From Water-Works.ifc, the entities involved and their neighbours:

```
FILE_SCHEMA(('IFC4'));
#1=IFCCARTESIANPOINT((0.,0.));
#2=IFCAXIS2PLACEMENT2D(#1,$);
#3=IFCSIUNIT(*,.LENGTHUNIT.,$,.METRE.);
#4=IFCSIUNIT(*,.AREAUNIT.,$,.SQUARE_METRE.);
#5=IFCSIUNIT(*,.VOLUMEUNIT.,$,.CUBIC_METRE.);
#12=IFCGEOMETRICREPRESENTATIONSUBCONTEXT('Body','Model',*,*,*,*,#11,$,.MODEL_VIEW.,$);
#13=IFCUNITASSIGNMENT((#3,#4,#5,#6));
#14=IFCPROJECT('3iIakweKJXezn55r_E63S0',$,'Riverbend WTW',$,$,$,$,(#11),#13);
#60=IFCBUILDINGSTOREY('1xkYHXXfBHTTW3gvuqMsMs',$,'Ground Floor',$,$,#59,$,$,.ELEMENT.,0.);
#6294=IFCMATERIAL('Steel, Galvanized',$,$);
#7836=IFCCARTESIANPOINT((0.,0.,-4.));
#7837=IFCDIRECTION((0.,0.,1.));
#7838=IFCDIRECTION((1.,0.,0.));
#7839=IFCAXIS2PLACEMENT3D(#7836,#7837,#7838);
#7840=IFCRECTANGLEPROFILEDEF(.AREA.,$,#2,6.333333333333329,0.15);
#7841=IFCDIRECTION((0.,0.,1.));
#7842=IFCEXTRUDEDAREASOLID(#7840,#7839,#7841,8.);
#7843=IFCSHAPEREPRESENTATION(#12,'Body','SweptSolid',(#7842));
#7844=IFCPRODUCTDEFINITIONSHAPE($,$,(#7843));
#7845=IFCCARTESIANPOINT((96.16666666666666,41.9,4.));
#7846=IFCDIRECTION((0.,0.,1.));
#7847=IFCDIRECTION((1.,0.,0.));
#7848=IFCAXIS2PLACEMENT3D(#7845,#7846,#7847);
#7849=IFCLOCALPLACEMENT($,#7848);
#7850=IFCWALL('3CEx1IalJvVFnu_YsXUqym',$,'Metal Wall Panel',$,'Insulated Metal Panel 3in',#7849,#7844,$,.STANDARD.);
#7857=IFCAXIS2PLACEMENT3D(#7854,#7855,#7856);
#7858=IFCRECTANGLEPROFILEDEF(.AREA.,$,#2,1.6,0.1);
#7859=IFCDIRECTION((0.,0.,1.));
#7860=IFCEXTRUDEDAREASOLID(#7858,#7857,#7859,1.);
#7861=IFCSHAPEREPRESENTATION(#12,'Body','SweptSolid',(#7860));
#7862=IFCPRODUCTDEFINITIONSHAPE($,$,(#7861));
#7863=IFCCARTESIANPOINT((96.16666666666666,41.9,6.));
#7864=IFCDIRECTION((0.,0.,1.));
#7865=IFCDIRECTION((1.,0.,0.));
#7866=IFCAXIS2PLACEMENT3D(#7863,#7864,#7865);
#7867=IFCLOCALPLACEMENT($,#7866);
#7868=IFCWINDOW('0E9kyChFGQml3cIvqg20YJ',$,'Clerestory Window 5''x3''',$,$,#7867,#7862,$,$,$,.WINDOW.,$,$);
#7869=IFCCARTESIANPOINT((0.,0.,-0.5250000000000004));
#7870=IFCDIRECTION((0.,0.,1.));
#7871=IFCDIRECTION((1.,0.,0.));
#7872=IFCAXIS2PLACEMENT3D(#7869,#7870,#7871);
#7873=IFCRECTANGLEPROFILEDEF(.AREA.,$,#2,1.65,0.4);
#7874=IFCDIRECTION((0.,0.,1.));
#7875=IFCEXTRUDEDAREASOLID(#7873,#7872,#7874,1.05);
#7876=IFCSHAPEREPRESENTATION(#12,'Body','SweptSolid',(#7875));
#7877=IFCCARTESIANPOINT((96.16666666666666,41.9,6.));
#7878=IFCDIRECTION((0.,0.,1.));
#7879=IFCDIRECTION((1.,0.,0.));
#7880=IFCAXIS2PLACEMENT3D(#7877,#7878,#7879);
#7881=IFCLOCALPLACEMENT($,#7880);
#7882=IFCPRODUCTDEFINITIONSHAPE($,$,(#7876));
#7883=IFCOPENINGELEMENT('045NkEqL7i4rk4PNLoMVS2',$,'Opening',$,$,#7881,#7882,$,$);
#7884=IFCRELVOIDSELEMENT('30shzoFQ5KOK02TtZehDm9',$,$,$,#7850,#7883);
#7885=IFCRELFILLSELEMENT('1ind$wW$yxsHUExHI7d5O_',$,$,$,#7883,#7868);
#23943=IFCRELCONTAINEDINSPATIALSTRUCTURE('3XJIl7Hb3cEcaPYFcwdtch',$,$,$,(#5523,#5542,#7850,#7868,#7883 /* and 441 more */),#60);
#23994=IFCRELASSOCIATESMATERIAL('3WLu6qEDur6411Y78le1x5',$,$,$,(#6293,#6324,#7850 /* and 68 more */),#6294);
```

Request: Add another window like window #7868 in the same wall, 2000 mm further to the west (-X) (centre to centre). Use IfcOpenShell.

```python
import ifcopenshell
import ifcopenshell.api.feature
import ifcopenshell.api.geometry
import ifcopenshell.api.root
import ifcopenshell.geom
import ifcopenshell.util.element
import ifcopenshell.util.placement
import ifcopenshell.util.shape

model = ifcopenshell.open("Water-Works.ifc")
settings = ifcopenshell.geom.settings()


def volume(element):
    """Net volume in cubic metres, openings subtracted."""
    shape = ifcopenshell.geom.create_shape(settings, element)
    return ifcopenshell.util.shape.get_volume(shape.geometry)


window = model.by_guid("0E9kyChFGQml3cIvqg20YJ")
opening = window.FillsVoids[0].RelatingOpeningElement
wall = opening.VoidsElements[0].RelatingBuildingElement
before = volume(wall)
shift = ifcopenshell.util.placement.get_local_placement(wall.ObjectPlacement)[:3, 0] * -2.0

# copy_class copies the void relationship, type, container and properties, but no geometry.
new_opening = ifcopenshell.api.root.copy_class(model, product=opening)
new_opening.Representation = ifcopenshell.util.element.copy_deep(
    model, opening.Representation, exclude=["IfcGeometricRepresentationContext", "IfcRepresentationMap"]
)
new_window = ifcopenshell.api.root.copy_class(model, product=window)
new_window.Representation = ifcopenshell.util.element.copy_deep(
    model, window.Representation, exclude=["IfcGeometricRepresentationContext", "IfcRepresentationMap"]
)
ifcopenshell.api.feature.add_filling(model, opening=new_opening, element=new_window)

for old, new in ((opening, new_opening), (window, new_window)):
    matrix = ifcopenshell.util.placement.get_local_placement(old.ObjectPlacement)
    matrix[:3, 3] += shift
    ifcopenshell.api.geometry.edit_object_placement(model, product=new, matrix=matrix, is_si=False)

after = volume(wall)

print(f"wall volume {before:.3f} -> {after:.3f} m3")

model.write("Water-Works_edited.ifc")
```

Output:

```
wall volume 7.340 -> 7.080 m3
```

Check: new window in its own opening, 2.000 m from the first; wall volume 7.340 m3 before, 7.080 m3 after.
